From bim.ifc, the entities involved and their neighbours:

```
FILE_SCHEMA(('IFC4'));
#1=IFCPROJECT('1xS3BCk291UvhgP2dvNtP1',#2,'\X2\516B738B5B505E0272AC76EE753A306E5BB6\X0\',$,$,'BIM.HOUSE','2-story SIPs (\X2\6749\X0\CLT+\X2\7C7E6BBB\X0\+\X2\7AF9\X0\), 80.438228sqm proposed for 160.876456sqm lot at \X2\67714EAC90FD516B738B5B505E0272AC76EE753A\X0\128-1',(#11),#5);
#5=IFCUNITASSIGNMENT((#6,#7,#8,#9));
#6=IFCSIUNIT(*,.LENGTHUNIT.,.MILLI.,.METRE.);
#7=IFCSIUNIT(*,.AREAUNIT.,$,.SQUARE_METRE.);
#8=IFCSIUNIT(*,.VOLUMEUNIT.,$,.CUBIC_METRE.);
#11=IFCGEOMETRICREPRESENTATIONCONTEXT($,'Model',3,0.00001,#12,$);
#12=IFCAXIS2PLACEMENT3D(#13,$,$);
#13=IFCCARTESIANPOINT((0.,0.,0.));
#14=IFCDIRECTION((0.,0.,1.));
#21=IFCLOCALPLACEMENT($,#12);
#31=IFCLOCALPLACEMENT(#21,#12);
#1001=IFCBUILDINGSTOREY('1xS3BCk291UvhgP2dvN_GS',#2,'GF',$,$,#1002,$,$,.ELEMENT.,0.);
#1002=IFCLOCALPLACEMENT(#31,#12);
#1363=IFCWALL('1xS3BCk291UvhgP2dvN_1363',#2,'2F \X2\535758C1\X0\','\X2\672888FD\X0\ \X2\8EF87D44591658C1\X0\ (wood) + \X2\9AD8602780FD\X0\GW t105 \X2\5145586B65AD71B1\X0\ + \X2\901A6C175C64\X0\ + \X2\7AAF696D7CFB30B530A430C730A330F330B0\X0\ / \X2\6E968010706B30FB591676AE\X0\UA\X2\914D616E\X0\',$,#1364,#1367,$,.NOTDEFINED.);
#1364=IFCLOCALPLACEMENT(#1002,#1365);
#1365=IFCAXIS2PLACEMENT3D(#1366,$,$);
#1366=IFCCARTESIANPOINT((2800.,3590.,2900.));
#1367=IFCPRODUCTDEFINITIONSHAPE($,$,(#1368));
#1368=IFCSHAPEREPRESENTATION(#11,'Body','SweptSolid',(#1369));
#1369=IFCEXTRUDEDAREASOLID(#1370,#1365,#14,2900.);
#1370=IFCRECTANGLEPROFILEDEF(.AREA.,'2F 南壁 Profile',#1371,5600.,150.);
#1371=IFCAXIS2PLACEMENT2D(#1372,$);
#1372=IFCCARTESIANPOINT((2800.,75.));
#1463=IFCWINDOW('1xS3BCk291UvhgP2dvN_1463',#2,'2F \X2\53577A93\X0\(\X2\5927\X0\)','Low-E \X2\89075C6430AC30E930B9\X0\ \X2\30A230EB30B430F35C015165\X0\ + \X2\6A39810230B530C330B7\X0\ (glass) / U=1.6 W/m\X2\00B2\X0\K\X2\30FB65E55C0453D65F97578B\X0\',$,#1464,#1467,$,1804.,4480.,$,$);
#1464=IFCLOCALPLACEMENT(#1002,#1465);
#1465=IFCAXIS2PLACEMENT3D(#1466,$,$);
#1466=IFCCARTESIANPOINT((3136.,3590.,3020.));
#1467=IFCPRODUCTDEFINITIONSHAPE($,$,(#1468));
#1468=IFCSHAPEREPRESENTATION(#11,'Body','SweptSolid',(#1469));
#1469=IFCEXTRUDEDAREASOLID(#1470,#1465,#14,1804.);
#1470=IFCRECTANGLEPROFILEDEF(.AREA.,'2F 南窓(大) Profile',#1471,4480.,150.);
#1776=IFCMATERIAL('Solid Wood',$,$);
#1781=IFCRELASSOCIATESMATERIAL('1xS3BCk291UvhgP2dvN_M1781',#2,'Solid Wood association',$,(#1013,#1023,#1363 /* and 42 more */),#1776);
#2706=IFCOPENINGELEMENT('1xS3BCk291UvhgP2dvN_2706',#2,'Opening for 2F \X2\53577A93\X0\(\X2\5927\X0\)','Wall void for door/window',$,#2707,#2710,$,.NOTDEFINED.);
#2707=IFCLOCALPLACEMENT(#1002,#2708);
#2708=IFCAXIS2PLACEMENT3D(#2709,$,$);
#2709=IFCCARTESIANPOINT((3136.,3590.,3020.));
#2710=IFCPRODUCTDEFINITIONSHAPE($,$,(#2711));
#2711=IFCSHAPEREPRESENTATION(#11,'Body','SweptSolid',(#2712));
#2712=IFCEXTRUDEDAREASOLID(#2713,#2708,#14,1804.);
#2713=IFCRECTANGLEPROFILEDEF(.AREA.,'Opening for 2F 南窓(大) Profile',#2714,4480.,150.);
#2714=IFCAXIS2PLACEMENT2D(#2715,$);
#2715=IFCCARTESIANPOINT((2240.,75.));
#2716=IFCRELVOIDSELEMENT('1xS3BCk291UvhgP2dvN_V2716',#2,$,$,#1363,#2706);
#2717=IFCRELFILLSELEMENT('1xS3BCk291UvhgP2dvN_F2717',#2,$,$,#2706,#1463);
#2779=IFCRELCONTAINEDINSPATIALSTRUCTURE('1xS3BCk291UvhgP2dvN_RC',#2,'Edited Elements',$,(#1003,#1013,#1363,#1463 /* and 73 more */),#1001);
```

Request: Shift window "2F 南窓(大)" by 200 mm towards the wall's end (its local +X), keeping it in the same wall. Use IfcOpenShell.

```python
import ifcopenshell
import ifcopenshell.api.geometry
import ifcopenshell.util.placement
import ifcopenshell.util.unit

model = ifcopenshell.open("bim.ifc")
unit_scale = ifcopenshell.util.unit.calculate_unit_scale(model)

window = model.by_id(1463)
opening = window.FillsVoids[0].RelatingOpeningElement
wall = opening.VoidsElements[0].RelatingBuildingElement

wall_matrix = ifcopenshell.util.placement.get_local_placement(wall.ObjectPlacement)
shift = wall_matrix[:3, 0] * 0.2 / unit_scale
before = ifcopenshell.util.placement.get_local_placement(window.ObjectPlacement)[:3, 3].copy()

# The window is not placed relative to its opening, so move both.
for product in (opening, window):
    matrix = ifcopenshell.util.placement.get_local_placement(product.ObjectPlacement)
    matrix[:3, 3] += shift
    ifcopenshell.api.geometry.edit_object_placement(model, product=product, matrix=matrix, is_si=False)

after = ifcopenshell.util.placement.get_local_placement(window.ObjectPlacement)[:3, 3]
print("window moved by", (after - before).round(3) + 0.0)

model.write("bim_rev.ifc")
```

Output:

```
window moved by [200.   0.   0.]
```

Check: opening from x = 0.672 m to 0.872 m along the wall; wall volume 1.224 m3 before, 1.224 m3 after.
